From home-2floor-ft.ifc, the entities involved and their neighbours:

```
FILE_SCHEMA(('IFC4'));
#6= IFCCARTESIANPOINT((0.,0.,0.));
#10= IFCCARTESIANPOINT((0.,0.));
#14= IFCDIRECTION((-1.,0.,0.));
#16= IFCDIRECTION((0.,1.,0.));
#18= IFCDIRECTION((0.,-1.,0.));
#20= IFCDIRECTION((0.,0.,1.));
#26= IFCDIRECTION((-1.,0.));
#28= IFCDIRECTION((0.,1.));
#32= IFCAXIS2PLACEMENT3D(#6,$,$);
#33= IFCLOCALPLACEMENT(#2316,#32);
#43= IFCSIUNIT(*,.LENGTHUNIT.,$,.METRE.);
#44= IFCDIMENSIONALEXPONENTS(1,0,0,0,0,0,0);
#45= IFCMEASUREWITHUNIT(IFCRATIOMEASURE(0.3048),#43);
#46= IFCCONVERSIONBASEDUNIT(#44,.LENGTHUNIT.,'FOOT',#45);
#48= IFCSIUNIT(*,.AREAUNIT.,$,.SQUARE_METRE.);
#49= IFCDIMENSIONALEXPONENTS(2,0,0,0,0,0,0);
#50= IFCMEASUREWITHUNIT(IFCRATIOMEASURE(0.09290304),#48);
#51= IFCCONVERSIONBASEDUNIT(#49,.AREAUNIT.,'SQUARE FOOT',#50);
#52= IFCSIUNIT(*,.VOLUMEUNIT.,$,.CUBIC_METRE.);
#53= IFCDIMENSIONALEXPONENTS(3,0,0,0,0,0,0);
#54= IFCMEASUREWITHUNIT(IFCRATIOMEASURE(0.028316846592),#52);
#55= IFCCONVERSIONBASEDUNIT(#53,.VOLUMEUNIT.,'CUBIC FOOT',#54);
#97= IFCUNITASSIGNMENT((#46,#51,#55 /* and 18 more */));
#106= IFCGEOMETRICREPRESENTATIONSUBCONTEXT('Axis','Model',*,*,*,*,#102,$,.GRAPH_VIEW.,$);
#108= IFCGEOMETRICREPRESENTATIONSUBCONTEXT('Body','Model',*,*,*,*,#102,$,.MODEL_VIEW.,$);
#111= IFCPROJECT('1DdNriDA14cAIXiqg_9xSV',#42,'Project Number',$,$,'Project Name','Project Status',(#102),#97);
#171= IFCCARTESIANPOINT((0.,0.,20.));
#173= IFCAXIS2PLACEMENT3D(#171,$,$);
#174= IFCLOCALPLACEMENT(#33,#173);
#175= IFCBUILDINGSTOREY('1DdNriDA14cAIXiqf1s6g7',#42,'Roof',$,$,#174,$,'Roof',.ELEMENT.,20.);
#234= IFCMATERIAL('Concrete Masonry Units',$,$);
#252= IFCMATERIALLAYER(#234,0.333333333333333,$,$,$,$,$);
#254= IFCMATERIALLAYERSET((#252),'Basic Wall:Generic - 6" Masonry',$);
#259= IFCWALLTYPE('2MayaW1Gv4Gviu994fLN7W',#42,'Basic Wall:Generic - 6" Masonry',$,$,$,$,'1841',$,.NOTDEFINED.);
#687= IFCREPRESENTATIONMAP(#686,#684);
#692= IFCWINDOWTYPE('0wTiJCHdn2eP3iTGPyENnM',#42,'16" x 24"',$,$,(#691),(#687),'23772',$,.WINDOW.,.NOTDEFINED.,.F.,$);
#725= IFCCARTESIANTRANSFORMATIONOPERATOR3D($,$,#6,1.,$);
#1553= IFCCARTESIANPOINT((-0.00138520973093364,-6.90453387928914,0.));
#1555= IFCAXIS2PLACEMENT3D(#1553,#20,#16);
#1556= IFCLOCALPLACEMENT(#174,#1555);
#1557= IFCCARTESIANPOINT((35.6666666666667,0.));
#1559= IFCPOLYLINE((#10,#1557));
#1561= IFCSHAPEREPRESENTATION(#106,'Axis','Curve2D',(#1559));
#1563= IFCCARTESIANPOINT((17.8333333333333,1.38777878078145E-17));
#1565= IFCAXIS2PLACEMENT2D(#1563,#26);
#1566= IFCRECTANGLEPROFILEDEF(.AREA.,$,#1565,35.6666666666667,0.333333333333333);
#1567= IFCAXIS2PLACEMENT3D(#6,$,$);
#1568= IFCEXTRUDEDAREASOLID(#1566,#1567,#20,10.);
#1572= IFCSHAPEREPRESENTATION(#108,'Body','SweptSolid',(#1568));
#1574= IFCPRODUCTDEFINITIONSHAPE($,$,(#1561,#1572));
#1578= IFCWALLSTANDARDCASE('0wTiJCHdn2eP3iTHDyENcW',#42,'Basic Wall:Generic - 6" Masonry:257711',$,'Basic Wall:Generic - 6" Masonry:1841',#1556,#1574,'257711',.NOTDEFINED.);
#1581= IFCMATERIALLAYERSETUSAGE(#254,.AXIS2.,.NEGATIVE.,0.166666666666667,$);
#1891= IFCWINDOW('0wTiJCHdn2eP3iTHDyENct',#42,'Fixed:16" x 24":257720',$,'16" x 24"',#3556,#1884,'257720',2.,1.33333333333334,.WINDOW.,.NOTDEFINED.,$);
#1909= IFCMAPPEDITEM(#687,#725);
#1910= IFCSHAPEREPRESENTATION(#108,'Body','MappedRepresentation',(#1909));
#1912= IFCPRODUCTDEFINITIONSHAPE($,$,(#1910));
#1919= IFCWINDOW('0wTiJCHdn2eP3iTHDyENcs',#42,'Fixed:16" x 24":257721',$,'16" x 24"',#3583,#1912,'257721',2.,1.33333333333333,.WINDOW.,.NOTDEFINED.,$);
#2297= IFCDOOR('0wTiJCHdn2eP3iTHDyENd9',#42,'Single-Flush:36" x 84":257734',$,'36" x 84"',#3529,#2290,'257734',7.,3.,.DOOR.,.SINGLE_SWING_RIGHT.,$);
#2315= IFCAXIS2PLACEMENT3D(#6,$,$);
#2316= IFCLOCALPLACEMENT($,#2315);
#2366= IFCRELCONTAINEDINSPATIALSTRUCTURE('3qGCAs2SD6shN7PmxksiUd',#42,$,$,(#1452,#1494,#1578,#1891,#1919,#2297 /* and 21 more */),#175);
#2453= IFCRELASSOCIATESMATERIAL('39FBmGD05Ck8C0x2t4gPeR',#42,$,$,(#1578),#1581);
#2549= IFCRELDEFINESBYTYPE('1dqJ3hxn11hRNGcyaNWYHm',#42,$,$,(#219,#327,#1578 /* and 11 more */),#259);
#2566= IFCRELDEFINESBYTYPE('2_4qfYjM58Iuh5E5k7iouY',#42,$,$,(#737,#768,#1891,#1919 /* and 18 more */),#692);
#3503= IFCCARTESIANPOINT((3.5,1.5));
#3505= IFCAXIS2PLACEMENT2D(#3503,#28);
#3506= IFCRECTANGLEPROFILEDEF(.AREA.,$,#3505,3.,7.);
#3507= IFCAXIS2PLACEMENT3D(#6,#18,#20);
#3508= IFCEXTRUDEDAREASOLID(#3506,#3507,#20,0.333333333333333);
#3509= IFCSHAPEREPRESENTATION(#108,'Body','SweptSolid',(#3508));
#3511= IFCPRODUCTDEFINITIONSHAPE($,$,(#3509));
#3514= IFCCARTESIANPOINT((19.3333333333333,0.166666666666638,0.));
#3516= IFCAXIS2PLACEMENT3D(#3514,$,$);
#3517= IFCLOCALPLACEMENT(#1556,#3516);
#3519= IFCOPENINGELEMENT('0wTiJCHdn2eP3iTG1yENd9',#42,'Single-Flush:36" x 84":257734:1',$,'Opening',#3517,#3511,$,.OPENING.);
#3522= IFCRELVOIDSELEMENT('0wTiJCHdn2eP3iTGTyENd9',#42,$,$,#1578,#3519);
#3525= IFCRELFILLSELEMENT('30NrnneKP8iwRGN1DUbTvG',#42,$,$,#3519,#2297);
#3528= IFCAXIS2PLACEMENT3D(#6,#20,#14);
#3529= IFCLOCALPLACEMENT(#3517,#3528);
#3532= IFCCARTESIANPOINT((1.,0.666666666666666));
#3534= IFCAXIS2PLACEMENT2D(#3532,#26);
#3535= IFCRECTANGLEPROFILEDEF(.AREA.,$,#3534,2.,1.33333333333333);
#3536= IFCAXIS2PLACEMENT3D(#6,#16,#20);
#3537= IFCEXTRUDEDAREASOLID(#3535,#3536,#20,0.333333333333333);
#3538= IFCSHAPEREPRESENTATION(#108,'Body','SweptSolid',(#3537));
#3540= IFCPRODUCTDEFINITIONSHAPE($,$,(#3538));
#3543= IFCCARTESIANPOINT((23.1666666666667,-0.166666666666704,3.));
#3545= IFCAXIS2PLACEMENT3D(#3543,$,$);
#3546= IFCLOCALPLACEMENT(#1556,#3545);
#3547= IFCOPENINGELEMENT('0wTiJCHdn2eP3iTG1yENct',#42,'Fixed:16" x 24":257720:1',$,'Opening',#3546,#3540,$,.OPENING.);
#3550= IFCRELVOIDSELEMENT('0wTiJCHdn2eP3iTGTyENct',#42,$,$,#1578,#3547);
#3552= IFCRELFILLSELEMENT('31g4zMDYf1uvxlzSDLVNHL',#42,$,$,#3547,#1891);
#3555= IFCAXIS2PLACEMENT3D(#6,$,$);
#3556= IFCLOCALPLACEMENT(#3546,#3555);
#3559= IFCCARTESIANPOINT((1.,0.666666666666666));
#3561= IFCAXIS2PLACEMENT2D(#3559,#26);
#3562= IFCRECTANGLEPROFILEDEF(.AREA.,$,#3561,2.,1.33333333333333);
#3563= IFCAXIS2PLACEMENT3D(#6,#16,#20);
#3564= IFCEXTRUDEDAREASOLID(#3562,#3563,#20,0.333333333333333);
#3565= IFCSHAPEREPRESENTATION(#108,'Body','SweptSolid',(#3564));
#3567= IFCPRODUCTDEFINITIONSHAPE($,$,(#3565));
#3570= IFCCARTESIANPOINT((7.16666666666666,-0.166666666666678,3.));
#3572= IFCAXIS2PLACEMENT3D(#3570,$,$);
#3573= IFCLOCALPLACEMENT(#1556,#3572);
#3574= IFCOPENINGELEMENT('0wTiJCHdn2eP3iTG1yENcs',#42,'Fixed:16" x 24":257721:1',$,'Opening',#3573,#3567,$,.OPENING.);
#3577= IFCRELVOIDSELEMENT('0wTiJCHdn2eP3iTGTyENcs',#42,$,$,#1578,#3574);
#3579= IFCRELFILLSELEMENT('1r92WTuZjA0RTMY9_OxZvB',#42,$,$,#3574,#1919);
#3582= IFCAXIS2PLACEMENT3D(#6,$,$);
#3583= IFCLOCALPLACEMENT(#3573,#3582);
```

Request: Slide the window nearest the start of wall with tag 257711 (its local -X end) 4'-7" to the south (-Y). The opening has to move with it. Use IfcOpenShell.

```python
import ifcopenshell
import ifcopenshell.api.geometry
import ifcopenshell.util.placement
import ifcopenshell.util.unit

model = ifcopenshell.open("home-2floor-ft.ifc")
unit_scale = ifcopenshell.util.unit.calculate_unit_scale(model)

window = model.by_guid("0wTiJCHdn2eP3iTHDyENcs")
opening = window.FillsVoids[0].RelatingOpeningElement
wall = opening.VoidsElements[0].RelatingBuildingElement

wall_matrix = ifcopenshell.util.placement.get_local_placement(wall.ObjectPlacement)
shift = wall_matrix[:3, 0] * -55 * 0.0254 / unit_scale
before = ifcopenshell.util.placement.get_local_placement(window.ObjectPlacement)[:3, 3].copy()

# The window is placed relative to its opening, so it follows when the opening moves.
matrix = ifcopenshell.util.placement.get_local_placement(opening.ObjectPlacement)
matrix[:3, 3] += shift
ifcopenshell.api.geometry.edit_object_placement(
    model, product=opening, matrix=matrix, is_si=False, should_transform_children=True
)

after = ifcopenshell.util.placement.get_local_placement(window.ObjectPlacement)[:3, 3]
print("window moved by", (after - before).round(3) + 0.0)

model.write("home-2floor-ft_rev.ifc")
```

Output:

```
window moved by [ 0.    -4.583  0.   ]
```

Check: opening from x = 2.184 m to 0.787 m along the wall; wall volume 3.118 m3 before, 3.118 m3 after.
